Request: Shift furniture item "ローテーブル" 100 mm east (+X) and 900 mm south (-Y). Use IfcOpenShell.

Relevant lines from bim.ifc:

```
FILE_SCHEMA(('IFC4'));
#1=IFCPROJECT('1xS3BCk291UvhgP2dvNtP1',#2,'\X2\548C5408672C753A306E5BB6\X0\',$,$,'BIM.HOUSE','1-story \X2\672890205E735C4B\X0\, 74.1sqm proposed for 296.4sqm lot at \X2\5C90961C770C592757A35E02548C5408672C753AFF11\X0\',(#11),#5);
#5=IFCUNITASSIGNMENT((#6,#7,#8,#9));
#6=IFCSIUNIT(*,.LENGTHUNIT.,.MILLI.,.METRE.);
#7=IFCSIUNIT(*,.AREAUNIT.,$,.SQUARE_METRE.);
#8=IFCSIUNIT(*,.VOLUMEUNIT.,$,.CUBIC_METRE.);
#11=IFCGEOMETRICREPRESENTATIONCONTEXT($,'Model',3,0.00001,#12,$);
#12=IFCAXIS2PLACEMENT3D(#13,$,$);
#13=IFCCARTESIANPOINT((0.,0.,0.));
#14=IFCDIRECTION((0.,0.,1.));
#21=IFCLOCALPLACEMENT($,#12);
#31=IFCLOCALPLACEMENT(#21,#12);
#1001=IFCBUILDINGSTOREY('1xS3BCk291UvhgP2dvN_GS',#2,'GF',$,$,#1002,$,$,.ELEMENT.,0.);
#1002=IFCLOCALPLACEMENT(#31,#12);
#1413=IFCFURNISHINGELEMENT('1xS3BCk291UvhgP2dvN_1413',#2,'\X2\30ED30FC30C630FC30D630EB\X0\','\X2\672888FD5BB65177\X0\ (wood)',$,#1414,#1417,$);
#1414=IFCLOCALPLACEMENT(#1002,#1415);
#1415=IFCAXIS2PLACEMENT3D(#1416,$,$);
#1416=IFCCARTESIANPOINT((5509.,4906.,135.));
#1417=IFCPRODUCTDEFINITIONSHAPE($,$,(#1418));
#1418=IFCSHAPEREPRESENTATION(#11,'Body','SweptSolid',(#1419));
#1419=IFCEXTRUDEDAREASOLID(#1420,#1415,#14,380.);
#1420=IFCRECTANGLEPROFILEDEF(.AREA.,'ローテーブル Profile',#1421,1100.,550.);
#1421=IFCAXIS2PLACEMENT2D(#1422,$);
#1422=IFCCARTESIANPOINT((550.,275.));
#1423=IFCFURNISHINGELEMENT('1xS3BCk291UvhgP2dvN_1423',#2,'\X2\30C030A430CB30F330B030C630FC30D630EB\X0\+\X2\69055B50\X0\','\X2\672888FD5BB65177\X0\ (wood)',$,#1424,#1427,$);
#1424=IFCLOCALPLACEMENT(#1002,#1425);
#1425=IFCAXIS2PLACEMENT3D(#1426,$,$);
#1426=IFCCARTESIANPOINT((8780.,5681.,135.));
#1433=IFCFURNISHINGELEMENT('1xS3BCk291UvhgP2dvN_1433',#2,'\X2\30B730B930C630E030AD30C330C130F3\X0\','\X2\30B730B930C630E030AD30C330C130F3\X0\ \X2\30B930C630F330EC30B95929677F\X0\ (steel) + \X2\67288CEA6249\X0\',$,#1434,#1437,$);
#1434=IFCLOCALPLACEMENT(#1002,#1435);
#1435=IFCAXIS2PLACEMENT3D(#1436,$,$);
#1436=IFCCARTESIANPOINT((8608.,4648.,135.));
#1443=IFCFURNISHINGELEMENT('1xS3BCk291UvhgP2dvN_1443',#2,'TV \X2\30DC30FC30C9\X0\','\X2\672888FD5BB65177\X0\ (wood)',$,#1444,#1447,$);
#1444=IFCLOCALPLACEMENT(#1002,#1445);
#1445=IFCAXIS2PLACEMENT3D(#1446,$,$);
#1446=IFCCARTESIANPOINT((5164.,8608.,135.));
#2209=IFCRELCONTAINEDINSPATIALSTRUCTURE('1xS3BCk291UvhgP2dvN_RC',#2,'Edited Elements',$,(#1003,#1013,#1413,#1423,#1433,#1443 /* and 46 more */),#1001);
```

```python
import ifcopenshell
import ifcopenshell.api.geometry
import ifcopenshell.util.placement
import ifcopenshell.util.unit

model = ifcopenshell.open("bim.ifc")
unit_scale = ifcopenshell.util.unit.calculate_unit_scale(model)

item = model.by_id(1413)
matrix = ifcopenshell.util.placement.get_local_placement(item.ObjectPlacement)
matrix[0, 3] += 0.1 / unit_scale
matrix[1, 3] -= 0.9 / unit_scale
ifcopenshell.api.geometry.edit_object_placement(model, product=item, matrix=matrix, is_si=False)

print(ifcopenshell.util.placement.get_local_placement(item.ObjectPlacement).round(3) + 0.0)

model.write("bim-out.ifc")
```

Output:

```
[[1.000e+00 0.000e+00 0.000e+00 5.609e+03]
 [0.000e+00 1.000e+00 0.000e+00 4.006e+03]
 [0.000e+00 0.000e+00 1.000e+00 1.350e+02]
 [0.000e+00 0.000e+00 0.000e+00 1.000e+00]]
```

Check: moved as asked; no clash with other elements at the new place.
